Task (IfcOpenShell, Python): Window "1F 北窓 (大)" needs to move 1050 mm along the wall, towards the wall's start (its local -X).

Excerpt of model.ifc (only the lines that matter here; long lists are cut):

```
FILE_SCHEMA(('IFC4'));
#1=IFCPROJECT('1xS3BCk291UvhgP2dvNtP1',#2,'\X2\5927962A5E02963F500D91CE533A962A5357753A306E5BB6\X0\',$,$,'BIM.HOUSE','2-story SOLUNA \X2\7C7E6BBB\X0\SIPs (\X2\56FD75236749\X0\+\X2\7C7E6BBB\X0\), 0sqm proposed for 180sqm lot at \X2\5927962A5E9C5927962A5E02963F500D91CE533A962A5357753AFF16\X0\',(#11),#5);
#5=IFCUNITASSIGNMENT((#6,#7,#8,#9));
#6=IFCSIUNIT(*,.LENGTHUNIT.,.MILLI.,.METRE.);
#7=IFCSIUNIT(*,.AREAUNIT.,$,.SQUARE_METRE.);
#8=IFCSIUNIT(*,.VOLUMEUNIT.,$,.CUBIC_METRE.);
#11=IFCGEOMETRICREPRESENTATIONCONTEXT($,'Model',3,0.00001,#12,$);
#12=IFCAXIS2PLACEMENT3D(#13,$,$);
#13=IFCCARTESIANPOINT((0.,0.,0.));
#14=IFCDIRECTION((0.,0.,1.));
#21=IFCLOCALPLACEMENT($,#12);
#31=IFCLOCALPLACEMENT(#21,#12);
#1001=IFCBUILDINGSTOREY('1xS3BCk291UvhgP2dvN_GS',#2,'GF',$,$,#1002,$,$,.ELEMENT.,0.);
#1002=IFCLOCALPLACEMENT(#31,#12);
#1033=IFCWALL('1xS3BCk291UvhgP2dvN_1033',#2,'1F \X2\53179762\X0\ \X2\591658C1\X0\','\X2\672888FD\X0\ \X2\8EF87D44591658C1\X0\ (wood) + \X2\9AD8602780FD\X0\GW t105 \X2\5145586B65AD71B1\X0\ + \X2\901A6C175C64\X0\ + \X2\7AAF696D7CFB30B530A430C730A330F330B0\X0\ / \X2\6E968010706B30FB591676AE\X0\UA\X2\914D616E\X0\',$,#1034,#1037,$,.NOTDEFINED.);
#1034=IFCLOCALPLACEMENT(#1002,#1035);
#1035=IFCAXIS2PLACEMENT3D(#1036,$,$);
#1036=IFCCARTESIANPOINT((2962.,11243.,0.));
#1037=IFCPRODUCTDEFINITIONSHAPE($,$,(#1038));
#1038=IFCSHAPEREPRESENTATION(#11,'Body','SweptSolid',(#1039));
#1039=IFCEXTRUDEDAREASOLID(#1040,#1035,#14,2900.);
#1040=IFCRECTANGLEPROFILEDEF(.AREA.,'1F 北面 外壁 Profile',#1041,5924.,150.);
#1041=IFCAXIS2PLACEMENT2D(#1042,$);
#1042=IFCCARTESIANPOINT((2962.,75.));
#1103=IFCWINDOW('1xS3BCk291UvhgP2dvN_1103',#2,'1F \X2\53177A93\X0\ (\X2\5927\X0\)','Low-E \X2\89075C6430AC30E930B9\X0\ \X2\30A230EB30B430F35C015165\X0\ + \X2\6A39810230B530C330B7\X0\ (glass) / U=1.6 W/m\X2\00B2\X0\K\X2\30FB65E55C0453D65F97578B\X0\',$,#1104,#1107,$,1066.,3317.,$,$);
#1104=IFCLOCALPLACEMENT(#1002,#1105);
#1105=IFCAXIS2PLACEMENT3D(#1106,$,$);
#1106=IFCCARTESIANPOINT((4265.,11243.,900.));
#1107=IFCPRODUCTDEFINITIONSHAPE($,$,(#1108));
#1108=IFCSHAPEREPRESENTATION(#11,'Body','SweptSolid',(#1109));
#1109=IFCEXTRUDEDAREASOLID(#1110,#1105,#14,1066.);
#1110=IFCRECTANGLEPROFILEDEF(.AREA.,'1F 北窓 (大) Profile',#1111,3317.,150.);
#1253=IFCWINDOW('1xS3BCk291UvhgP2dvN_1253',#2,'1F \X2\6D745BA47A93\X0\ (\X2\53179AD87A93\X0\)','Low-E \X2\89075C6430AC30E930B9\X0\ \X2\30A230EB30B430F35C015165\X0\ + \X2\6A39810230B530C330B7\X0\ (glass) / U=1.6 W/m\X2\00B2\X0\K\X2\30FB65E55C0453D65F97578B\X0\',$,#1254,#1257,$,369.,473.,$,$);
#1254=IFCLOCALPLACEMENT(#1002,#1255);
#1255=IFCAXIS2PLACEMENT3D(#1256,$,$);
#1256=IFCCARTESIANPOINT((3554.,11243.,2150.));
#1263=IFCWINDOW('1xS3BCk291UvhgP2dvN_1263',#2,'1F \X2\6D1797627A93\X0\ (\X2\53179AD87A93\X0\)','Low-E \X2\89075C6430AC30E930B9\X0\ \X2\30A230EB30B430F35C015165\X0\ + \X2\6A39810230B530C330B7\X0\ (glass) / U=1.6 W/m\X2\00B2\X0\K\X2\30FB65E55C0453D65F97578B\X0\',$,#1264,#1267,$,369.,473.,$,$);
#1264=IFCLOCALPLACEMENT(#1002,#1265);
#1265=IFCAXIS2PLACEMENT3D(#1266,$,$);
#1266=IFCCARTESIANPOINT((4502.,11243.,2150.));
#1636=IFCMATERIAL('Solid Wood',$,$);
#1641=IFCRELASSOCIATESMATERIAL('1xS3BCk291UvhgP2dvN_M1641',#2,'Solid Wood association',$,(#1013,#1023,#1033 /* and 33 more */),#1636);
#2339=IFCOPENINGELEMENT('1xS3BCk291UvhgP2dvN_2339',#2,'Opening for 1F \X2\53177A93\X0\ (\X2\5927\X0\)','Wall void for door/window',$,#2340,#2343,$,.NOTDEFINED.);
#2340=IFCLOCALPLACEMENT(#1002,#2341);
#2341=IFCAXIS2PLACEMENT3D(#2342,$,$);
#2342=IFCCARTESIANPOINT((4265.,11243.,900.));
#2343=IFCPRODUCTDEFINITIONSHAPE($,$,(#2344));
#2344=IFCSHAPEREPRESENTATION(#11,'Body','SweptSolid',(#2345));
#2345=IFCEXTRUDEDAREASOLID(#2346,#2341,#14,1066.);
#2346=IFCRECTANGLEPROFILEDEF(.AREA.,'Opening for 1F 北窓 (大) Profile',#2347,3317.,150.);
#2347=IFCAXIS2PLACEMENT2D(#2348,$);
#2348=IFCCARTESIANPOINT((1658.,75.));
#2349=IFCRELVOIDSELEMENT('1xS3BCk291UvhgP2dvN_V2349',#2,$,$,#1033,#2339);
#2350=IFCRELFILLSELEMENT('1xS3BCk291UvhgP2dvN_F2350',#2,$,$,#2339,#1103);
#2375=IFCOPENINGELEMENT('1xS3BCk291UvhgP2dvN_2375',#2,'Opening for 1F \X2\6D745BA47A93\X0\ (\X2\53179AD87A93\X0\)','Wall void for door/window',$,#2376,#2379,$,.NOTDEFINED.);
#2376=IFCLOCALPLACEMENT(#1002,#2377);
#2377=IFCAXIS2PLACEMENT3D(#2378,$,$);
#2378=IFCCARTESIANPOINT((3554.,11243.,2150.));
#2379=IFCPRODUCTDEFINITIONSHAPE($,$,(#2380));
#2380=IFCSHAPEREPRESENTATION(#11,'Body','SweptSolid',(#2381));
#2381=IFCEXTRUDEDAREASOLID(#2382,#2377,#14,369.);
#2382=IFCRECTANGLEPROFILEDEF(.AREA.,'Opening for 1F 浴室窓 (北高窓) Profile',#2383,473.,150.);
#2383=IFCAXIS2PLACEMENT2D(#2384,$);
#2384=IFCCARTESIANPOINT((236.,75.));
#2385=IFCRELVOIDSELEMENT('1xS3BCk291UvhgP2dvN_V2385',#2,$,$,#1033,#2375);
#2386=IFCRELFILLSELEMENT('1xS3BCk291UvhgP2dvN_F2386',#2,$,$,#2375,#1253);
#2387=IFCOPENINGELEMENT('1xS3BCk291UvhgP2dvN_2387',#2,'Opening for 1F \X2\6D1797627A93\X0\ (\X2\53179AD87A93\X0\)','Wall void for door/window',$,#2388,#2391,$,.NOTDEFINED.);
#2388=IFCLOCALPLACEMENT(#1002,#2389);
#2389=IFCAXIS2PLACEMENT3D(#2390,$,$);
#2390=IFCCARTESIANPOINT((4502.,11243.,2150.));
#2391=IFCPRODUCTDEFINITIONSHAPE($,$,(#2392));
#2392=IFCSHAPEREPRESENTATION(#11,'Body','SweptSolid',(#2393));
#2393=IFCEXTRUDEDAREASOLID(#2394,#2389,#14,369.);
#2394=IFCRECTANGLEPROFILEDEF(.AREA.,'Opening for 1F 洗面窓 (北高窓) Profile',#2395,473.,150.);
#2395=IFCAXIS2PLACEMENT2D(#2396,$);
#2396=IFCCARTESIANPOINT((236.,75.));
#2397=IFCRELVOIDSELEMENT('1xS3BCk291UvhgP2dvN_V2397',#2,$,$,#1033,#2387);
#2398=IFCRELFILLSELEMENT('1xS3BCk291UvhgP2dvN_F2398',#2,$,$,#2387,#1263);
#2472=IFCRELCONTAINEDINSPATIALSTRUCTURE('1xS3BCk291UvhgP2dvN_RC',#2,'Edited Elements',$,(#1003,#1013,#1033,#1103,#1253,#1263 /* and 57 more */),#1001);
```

```python
import ifcopenshell
import ifcopenshell.api.geometry
import ifcopenshell.util.placement
import ifcopenshell.util.unit

model = ifcopenshell.open("model.ifc")
unit_scale = ifcopenshell.util.unit.calculate_unit_scale(model)

window = model.by_guid("1xS3BCk291UvhgP2dvN_1103")
opening = window.FillsVoids[0].RelatingOpeningElement
wall = opening.VoidsElements[0].RelatingBuildingElement

wall_matrix = ifcopenshell.util.placement.get_local_placement(wall.ObjectPlacement)
shift = wall_matrix[:3, 0] * -1.05 / unit_scale
before = ifcopenshell.util.placement.get_local_placement(window.ObjectPlacement)[:3, 3].copy()

# The window is not placed relative to its opening, so move both.
for product in (opening, window):
    matrix = ifcopenshell.util.placement.get_local_placement(product.ObjectPlacement)
    matrix[:3, 3] += shift
    ifcopenshell.api.geometry.edit_object_placement(model, product=product, matrix=matrix, is_si=False)

after = ifcopenshell.util.placement.get_local_placement(window.ObjectPlacement)[:3, 3]
print("window moved by", (after - before).round(3) + 0.0)

model.write("model_updated.ifc")
```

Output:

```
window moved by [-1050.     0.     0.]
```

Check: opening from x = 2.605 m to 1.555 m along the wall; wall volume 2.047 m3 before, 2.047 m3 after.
